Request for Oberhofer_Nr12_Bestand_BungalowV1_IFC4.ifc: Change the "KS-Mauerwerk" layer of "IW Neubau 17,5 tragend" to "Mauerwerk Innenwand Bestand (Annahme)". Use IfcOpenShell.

First a look at what the model holds.

```python
import ifcopenshell
import ifcopenshell.util.element

model = ifcopenshell.open("Oberhofer_Nr12_Bestand_BungalowV1_IFC4.ifc")
print(model.schema)
for layer_set in model.by_type("IfcMaterialLayerSet"):
    if layer_set.LayerSetName == "IW Neubau 17,5 tragend":
        for layer in layer_set.MaterialLayers:
            print(layer.id(), layer.Material and layer.Material.Name, layer.LayerThickness, sep=" | ")
        print(len(ifcopenshell.util.element.get_elements_by_material(model, layer_set)), "elements and types use it")
print(sorted(m.Name for m in model.by_type("IfcMaterial") if m.Name)[:60])
```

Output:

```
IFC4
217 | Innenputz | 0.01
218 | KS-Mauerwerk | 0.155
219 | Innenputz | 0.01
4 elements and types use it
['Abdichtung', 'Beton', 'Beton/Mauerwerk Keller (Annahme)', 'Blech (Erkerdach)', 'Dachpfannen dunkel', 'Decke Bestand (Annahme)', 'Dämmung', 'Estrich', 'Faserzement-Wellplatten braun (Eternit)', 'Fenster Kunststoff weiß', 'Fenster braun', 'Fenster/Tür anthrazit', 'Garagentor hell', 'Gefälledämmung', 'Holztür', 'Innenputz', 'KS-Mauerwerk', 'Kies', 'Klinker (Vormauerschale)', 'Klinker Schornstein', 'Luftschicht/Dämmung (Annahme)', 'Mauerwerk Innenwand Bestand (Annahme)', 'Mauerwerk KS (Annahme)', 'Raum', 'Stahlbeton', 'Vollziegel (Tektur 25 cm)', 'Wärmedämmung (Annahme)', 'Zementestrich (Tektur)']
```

```python
import ifcopenshell
import ifcopenshell.api.material

model = ifcopenshell.open("Oberhofer_Nr12_Bestand_BungalowV1_IFC4.ifc")

layer_set = next(s for s in model.by_type("IfcMaterialLayerSet") if s.LayerSetName == "IW Neubau 17,5 tragend")
layer = next(l for l in layer_set.MaterialLayers if l.Material and l.Material.Name == "KS-Mauerwerk")
material = next(m for m in model.by_type("IfcMaterial") if m.Name == "Mauerwerk Innenwand Bestand (Annahme)")

# Point this one layer at the other material; renaming the old one would change it everywhere.
ifcopenshell.api.material.edit_layer(model, layer=layer, attributes={}, material=material)

print([l.Material.Name if l.Material else None for l in layer_set.MaterialLayers])

model.write("Oberhofer_Nr12_Bestand_BungalowV1_IFC4-out.ifc")
```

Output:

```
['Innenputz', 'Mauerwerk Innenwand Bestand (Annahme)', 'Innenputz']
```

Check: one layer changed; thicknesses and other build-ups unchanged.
